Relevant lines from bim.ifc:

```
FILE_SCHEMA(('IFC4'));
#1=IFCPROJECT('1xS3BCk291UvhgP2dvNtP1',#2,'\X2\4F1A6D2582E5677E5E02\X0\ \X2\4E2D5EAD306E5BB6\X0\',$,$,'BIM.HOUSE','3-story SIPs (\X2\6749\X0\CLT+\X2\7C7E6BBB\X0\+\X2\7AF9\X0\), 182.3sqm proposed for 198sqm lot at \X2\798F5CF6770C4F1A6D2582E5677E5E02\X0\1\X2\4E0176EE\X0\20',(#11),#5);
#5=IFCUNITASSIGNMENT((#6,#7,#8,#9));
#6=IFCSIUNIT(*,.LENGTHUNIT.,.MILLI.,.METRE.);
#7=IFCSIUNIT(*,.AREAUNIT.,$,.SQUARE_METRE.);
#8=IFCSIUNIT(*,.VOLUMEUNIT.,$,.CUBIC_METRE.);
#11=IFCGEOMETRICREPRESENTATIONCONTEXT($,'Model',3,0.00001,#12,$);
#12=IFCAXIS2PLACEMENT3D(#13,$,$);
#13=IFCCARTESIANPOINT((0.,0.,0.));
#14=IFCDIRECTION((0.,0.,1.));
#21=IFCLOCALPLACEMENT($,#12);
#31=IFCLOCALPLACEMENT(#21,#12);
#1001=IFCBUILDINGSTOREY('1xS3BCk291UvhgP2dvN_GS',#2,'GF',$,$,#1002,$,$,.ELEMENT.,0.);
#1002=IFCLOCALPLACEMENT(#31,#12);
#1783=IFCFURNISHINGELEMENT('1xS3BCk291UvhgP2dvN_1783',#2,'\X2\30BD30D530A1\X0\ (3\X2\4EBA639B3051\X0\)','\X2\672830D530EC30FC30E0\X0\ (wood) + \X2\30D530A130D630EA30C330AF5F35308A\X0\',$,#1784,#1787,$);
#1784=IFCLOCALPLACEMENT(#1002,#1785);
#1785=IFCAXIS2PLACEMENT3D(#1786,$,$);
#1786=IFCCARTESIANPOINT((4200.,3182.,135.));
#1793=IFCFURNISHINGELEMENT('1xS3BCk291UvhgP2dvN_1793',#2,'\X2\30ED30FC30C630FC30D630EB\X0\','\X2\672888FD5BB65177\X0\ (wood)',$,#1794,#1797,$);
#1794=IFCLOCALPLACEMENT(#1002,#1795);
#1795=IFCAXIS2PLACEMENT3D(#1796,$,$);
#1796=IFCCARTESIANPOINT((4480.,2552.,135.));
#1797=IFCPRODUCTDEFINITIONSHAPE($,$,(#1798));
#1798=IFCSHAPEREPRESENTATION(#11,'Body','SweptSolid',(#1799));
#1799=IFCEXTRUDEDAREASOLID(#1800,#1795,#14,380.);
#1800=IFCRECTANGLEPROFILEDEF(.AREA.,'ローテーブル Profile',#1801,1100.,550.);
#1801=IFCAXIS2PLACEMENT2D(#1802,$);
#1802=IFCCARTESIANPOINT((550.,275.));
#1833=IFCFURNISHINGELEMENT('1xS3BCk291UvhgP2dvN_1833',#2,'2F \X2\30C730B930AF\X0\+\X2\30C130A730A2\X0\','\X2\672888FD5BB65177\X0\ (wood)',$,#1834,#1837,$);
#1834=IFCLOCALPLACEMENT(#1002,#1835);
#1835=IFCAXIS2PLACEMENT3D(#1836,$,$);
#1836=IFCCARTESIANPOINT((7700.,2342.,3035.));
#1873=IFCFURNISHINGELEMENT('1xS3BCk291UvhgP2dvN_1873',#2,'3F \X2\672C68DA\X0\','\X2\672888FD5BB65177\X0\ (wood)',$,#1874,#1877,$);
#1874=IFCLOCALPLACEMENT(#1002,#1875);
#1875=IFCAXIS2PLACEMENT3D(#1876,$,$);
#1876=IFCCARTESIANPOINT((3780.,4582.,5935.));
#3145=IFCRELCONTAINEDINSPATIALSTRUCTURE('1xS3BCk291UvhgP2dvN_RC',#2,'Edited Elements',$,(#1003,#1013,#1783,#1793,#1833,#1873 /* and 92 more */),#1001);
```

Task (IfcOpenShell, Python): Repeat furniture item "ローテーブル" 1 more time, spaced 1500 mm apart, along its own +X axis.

```python
import ifcopenshell
import ifcopenshell.api.geometry
import ifcopenshell.api.root
import ifcopenshell.util.element
import ifcopenshell.util.placement

model = ifcopenshell.open("bim.ifc")


def reuse_history(source, copy):
    """copy_class also copies each property set's owner history, people and application; keep the originals."""
    for rel in copy.IsDefinedBy:
        if rel.is_a("IfcRelDefinesByProperties") and (history := rel.RelatingPropertyDefinition.OwnerHistory):
            rel.RelatingPropertyDefinition.OwnerHistory = source.OwnerHistory
            ifcopenshell.util.element.remove_deep2(model, history)


source = model.by_guid("1xS3BCk291UvhgP2dvN_1793")
base = ifcopenshell.util.placement.get_local_placement(source.ObjectPlacement)
step = base[:3, 0] * 1500.0

for i in range(1, 2):
    copy = ifcopenshell.api.root.copy_class(model, product=source)
    copy.Representation = ifcopenshell.util.element.copy_deep(
        model, source.Representation, exclude=["IfcGeometricRepresentationContext", "IfcRepresentationMap"]
    )
    reuse_history(source, copy)
    matrix = base.copy()
    matrix[:3, 3] += i * step
    print("added at", matrix[:3, 3].round(3) + 0.0)
    ifcopenshell.api.geometry.edit_object_placement(model, product=copy, matrix=matrix, is_si=False)

model.write("bim-out.ifc")
```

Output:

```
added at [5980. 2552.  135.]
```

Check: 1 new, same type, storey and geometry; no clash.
